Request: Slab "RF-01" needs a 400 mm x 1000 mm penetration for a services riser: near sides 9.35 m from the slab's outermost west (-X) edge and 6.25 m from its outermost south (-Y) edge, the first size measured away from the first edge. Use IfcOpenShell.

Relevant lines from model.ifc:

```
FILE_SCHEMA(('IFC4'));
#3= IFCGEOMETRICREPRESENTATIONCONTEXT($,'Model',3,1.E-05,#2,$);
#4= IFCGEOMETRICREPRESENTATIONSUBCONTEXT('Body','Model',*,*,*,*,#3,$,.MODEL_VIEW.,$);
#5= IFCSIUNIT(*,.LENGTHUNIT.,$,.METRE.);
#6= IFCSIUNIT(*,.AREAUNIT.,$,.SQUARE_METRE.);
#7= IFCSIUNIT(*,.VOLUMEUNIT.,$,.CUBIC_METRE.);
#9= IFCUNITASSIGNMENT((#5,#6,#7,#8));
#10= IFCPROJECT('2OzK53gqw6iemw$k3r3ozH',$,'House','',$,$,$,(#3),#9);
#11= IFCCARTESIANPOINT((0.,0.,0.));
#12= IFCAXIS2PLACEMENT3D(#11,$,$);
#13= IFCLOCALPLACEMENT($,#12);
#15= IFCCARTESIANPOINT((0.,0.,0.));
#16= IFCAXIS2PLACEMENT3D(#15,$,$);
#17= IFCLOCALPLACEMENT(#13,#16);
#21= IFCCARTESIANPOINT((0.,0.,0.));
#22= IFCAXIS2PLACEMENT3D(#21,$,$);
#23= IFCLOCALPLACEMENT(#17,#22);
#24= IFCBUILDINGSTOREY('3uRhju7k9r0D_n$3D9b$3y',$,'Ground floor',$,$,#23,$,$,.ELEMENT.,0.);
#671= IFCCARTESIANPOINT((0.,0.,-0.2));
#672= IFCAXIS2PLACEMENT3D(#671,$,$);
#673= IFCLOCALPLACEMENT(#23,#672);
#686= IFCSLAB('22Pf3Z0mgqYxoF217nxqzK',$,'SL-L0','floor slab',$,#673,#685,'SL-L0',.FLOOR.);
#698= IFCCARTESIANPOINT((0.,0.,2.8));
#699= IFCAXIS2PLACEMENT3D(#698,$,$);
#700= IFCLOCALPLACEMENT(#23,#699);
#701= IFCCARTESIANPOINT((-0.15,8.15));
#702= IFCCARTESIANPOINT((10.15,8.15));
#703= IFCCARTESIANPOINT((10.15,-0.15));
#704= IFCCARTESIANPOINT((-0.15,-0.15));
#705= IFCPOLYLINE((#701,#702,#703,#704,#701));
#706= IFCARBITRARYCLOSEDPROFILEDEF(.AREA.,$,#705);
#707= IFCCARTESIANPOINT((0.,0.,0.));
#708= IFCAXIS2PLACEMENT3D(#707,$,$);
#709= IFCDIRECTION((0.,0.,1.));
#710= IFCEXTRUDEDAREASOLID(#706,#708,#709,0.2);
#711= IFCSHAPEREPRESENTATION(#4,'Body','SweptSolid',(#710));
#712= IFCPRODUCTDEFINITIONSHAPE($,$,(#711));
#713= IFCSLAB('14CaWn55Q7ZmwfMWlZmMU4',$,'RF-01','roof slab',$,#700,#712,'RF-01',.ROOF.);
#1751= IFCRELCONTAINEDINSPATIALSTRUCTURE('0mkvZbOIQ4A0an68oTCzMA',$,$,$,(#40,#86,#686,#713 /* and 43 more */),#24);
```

```python
import numpy as np
import ifcopenshell
import ifcopenshell.api.feature
import ifcopenshell.api.geometry
import ifcopenshell.api.root
import ifcopenshell.geom
import ifcopenshell.util.placement
import ifcopenshell.util.representation
import ifcopenshell.util.shape
import ifcopenshell.util.unit

model = ifcopenshell.open("model.ifc")
unit_scale = ifcopenshell.util.unit.calculate_unit_scale(model)
settings = ifcopenshell.geom.settings()


def volume(element):
    """Net volume in cubic metres, openings subtracted."""
    shape = ifcopenshell.geom.create_shape(settings, element)
    return ifcopenshell.util.shape.get_volume(shape.geometry)


slab = model.by_id(713)
before = volume(slab)

# Extent in the slab's own axes, in metres. The edges named are its -X and -Y sides.
slab_shape = ifcopenshell.geom.create_shape(settings, slab)
vertices = ifcopenshell.util.shape.get_vertices(slab_shape.geometry)
x_min, y_min, bottom = vertices.min(axis=0)
top = vertices[:, 2].max()

opening = ifcopenshell.api.root.create_entity(model, ifc_class="IfcOpeningElement", name="Services riser opening", predefined_type="OPENING")
context = ifcopenshell.util.representation.get_context(model, "Model", "Body", "MODEL_VIEW")
width, depth = 0.4, 1
outline = [(0.0, 0.0), (width, 0.0), (width, depth), (0.0, depth), (0.0, 0.0)]
# Overshoot both faces by 50 mm so the cut is clean.
shape = ifcopenshell.api.geometry.add_slab_representation(
    model, context=context, depth=top - bottom + 0.1, polyline=outline
)
ifcopenshell.api.geometry.assign_representation(model, product=opening, representation=shape)

matrix = ifcopenshell.util.placement.get_local_placement(slab.ObjectPlacement)
matrix[:, 3] = matrix @ np.append(np.array([x_min + 9.35, y_min + 6.25, bottom - 0.05]) / unit_scale, 1.0)
ifcopenshell.api.geometry.edit_object_placement(model, product=opening, matrix=matrix, is_si=False)
ifcopenshell.api.feature.add_feature(model, feature=opening, element=slab)

after = volume(slab)

print(f"slab volume {before:.3f} -> {after:.3f} m3")

model.write("model_edited.ifc")
```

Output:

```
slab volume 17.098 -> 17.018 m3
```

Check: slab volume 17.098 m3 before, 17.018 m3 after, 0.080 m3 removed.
